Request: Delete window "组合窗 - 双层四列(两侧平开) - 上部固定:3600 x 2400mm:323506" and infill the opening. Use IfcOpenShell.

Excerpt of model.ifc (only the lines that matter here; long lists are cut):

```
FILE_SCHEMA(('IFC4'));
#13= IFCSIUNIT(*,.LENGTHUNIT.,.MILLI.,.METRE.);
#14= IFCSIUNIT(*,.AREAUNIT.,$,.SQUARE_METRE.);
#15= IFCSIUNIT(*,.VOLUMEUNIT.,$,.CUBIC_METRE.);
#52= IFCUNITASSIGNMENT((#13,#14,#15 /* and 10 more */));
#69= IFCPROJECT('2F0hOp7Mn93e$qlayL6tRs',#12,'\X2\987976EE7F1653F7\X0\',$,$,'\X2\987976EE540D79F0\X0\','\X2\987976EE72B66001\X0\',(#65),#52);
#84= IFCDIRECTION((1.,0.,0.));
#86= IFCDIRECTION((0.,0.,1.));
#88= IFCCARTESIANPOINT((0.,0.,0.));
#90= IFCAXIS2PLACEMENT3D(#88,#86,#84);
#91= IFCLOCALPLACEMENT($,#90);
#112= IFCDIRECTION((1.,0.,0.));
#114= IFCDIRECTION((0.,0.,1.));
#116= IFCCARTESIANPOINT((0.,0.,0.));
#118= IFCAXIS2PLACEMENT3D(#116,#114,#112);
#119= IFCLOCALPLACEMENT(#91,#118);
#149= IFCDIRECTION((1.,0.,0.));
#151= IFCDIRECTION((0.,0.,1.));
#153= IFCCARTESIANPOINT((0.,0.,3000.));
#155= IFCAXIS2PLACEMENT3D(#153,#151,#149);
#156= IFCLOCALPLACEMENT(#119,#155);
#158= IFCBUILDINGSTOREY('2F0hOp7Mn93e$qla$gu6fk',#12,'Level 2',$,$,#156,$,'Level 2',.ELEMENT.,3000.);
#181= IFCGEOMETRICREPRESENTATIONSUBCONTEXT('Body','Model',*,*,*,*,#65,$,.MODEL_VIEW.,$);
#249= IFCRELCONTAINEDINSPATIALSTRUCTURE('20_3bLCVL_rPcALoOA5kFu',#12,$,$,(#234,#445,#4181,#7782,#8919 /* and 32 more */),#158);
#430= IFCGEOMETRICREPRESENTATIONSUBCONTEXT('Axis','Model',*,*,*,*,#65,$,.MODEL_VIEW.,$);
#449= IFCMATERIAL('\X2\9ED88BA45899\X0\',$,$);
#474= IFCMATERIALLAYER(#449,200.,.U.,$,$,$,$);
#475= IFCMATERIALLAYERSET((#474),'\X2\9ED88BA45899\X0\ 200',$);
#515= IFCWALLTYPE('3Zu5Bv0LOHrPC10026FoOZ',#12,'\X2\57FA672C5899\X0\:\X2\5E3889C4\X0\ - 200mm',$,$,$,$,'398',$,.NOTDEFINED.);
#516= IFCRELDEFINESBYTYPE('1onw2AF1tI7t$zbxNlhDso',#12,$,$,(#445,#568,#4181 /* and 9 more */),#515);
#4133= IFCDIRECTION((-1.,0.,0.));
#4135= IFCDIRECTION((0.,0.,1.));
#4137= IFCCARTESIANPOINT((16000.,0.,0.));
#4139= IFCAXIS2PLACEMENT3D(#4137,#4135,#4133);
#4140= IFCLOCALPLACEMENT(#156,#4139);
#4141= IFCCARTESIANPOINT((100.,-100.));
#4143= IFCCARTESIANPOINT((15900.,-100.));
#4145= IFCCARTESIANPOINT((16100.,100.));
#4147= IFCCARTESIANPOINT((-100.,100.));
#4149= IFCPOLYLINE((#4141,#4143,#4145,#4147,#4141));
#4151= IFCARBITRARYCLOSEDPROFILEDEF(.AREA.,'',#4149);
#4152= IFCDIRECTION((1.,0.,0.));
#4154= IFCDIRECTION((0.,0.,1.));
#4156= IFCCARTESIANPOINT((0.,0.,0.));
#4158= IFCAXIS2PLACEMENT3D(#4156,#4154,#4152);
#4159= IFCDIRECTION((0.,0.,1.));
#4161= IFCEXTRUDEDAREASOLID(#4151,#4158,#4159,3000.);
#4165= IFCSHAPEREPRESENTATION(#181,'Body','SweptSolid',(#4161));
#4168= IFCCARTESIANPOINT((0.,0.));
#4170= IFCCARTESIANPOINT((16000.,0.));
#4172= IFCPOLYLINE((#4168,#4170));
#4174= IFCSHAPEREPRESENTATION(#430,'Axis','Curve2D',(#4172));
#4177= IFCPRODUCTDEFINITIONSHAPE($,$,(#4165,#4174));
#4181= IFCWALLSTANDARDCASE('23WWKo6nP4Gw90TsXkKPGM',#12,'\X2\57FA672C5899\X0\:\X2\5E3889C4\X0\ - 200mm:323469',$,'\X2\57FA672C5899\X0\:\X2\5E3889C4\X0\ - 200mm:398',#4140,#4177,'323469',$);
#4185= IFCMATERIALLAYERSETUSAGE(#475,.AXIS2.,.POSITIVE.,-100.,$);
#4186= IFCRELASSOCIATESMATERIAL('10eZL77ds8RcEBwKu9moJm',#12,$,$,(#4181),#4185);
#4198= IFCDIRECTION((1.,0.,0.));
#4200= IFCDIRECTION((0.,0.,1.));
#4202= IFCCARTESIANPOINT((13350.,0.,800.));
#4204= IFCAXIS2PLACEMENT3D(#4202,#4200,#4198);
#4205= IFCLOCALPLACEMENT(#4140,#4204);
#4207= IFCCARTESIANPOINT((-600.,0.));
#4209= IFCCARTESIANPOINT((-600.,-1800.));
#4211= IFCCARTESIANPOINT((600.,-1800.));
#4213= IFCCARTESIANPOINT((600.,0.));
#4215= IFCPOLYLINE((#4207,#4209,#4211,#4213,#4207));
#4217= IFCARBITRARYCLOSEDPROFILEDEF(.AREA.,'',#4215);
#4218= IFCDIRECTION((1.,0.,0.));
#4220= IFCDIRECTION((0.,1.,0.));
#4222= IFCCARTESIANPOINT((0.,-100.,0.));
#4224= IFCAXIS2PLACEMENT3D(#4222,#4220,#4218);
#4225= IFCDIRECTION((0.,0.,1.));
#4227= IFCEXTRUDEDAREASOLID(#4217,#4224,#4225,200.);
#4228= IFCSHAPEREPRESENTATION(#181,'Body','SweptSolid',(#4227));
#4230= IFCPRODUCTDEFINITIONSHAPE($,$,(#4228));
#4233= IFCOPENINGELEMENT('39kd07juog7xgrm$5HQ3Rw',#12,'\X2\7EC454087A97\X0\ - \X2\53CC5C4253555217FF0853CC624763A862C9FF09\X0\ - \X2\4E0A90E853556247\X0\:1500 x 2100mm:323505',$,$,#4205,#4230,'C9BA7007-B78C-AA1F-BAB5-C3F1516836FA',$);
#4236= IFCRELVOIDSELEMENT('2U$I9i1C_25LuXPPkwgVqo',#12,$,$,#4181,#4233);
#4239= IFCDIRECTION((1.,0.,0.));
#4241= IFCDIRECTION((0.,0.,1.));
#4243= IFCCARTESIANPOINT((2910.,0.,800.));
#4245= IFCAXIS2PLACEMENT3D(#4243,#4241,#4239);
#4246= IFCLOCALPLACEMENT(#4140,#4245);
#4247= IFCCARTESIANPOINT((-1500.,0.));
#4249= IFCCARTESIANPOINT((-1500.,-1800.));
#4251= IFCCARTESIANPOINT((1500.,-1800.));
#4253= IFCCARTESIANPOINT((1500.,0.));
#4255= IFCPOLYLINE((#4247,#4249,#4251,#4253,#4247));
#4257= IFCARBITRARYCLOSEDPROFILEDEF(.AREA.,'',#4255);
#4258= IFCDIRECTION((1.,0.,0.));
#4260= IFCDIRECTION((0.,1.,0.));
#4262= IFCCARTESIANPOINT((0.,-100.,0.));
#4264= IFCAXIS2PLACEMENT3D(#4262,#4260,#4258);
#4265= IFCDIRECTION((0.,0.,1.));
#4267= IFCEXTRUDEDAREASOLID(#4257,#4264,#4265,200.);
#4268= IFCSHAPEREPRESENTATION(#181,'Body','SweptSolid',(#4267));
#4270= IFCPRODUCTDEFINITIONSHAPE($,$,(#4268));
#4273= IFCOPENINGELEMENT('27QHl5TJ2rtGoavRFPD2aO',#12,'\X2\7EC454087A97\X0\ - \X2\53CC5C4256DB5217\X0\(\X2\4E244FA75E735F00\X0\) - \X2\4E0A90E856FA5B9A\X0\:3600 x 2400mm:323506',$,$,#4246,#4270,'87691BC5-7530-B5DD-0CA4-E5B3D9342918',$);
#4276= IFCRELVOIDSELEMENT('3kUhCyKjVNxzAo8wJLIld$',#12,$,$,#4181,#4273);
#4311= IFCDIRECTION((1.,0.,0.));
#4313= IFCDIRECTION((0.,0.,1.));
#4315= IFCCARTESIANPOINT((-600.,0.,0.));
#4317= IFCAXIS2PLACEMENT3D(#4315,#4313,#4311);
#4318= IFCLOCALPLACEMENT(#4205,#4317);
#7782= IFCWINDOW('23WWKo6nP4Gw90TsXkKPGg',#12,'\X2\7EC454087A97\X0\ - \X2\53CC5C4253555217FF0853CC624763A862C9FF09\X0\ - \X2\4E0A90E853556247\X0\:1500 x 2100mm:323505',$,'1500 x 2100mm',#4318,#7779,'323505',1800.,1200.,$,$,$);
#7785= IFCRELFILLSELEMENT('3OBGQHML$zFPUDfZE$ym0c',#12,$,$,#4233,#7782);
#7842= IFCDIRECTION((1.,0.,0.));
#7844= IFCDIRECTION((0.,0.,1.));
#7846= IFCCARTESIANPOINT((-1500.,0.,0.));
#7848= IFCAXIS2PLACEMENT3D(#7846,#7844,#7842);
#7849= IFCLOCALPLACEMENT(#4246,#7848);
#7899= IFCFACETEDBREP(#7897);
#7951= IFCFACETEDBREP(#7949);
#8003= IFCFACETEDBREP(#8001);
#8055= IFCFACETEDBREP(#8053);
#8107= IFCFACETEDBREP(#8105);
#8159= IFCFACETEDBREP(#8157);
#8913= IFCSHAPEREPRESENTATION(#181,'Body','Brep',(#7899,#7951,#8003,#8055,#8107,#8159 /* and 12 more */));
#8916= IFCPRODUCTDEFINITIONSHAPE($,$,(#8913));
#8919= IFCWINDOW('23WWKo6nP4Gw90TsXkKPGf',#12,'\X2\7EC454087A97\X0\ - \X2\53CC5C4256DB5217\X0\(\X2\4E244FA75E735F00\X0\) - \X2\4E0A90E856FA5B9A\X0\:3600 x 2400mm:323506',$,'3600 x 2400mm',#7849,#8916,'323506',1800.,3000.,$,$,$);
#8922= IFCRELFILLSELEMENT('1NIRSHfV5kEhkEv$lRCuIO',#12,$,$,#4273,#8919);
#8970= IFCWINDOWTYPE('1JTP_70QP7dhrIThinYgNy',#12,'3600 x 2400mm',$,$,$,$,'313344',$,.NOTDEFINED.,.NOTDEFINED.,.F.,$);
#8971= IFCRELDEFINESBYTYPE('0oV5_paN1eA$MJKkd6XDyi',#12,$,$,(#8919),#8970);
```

```python
import ifcopenshell
import ifcopenshell.api.feature
import ifcopenshell.api.root
import ifcopenshell.geom
import ifcopenshell.util.shape

model = ifcopenshell.open("model.ifc")
settings = ifcopenshell.geom.settings()


def volume(element):
    """Net volume in cubic metres, openings subtracted."""
    shape = ifcopenshell.geom.create_shape(settings, element)
    return ifcopenshell.util.shape.get_volume(shape.geometry)


window = model.by_guid("23WWKo6nP4Gw90TsXkKPGf")
opening = window.FillsVoids[0].RelatingOpeningElement
wall = opening.VoidsElements[0].RelatingBuildingElement
before = volume(wall)

ifcopenshell.api.root.remove_product(model, product=window)
ifcopenshell.api.feature.remove_feature(model, feature=opening)

after = volume(wall)

print(f"wall volume {before:.3f} -> {after:.3f} m3")

model.write("model_v2.ifc")
```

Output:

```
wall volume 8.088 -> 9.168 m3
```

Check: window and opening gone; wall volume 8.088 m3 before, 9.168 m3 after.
